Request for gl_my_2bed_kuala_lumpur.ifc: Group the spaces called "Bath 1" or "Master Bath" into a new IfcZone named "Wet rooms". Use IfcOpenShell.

First a look at what the model holds.

```python
import ifcopenshell

model = ifcopenshell.open("gl_my_2bed_kuala_lumpur.ifc")
print(model.schema)
seen = {}
for space in model.by_type("IfcSpace"):
    seen[space.LongName] = seen.get(space.LongName, 0) + 1
for name, count in sorted(seen.items(), key=str):
    print(count, "x", name)
print("zones:", [z.Name for z in model.by_type("IfcZone")][:20])
```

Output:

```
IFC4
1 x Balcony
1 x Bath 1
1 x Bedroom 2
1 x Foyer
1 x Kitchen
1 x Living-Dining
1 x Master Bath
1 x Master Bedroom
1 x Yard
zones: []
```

```python
import ifcopenshell
import ifcopenshell.api.group
import ifcopenshell.api.root

model = ifcopenshell.open("gl_my_2bed_kuala_lumpur.ifc")

names = {"Bath 1", "Master Bath"}
spaces = [s for s in model.by_type("IfcSpace") if s.LongName in names]

zone = ifcopenshell.api.root.create_entity(model, ifc_class="IfcZone", name="Wet rooms")
ifcopenshell.api.group.assign_group(model, products=spaces, group=zone)
print(len(spaces), "spaces in", zone.Name)

model.write("gl_my_2bed_kuala_lumpur-out.ifc")
```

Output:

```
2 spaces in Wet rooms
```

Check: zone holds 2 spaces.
